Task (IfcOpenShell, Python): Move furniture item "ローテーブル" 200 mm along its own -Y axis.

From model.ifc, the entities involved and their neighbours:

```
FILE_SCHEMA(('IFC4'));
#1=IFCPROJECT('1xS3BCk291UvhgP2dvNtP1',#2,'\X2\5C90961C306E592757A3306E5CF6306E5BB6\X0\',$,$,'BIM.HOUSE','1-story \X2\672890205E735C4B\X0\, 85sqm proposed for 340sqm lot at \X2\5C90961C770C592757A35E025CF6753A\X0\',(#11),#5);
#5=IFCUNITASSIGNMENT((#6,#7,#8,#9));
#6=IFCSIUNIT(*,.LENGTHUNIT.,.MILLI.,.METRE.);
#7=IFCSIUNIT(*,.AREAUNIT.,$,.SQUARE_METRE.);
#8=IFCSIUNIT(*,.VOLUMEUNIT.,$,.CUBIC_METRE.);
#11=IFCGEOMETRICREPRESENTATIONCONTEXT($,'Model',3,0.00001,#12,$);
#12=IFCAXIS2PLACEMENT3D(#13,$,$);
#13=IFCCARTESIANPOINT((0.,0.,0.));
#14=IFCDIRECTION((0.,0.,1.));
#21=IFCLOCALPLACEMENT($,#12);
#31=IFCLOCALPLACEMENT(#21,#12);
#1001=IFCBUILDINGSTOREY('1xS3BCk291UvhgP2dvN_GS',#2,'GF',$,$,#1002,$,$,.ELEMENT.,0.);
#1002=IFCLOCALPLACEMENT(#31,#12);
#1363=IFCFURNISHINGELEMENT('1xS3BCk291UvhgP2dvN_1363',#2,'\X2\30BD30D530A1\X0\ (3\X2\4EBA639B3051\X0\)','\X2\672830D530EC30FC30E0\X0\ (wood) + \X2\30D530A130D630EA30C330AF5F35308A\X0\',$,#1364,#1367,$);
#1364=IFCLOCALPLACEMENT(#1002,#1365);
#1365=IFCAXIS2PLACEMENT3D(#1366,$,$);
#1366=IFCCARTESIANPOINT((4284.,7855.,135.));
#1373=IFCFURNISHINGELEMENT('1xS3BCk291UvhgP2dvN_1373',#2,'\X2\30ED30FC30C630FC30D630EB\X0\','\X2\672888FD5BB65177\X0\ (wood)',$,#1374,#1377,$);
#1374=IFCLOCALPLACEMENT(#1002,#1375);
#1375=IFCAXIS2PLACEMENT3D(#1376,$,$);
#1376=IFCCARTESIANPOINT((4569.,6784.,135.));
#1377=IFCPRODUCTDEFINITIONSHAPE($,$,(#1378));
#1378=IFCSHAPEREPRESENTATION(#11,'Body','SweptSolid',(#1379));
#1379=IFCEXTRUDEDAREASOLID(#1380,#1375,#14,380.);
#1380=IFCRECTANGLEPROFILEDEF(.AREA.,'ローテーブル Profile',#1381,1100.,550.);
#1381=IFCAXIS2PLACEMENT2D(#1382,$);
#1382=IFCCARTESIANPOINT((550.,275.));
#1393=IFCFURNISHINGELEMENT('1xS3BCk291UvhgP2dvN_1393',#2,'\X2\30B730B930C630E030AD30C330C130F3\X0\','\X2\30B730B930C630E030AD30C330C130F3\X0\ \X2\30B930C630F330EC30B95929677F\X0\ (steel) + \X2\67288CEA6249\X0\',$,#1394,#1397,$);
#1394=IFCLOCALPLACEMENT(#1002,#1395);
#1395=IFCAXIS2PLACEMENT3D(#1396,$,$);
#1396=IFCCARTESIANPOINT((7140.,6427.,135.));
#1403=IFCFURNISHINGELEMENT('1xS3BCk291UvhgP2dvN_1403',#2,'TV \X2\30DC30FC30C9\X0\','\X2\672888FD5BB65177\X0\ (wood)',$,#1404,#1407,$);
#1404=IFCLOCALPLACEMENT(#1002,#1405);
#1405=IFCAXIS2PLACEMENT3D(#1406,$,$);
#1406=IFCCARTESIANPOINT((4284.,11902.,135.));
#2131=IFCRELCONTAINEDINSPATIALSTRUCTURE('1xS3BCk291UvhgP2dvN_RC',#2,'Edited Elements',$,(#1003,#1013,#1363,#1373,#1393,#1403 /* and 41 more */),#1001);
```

```python
import ifcopenshell
import ifcopenshell.api.geometry
import ifcopenshell.util.placement
import ifcopenshell.util.unit

model = ifcopenshell.open("model.ifc")
unit_scale = ifcopenshell.util.unit.calculate_unit_scale(model)

item = model.by_guid("1xS3BCk291UvhgP2dvN_1373")
matrix = ifcopenshell.util.placement.get_local_placement(item.ObjectPlacement)
matrix[:3, 3] -= matrix[:3, 1] * 0.2 / unit_scale
ifcopenshell.api.geometry.edit_object_placement(model, product=item, matrix=matrix, is_si=False)

print(ifcopenshell.util.placement.get_local_placement(item.ObjectPlacement).round(3) + 0.0)

model.write("model-out.ifc")
```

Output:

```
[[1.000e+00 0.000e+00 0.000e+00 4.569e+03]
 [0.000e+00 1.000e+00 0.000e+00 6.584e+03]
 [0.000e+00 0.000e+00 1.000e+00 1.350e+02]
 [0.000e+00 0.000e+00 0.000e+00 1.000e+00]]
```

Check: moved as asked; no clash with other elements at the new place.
